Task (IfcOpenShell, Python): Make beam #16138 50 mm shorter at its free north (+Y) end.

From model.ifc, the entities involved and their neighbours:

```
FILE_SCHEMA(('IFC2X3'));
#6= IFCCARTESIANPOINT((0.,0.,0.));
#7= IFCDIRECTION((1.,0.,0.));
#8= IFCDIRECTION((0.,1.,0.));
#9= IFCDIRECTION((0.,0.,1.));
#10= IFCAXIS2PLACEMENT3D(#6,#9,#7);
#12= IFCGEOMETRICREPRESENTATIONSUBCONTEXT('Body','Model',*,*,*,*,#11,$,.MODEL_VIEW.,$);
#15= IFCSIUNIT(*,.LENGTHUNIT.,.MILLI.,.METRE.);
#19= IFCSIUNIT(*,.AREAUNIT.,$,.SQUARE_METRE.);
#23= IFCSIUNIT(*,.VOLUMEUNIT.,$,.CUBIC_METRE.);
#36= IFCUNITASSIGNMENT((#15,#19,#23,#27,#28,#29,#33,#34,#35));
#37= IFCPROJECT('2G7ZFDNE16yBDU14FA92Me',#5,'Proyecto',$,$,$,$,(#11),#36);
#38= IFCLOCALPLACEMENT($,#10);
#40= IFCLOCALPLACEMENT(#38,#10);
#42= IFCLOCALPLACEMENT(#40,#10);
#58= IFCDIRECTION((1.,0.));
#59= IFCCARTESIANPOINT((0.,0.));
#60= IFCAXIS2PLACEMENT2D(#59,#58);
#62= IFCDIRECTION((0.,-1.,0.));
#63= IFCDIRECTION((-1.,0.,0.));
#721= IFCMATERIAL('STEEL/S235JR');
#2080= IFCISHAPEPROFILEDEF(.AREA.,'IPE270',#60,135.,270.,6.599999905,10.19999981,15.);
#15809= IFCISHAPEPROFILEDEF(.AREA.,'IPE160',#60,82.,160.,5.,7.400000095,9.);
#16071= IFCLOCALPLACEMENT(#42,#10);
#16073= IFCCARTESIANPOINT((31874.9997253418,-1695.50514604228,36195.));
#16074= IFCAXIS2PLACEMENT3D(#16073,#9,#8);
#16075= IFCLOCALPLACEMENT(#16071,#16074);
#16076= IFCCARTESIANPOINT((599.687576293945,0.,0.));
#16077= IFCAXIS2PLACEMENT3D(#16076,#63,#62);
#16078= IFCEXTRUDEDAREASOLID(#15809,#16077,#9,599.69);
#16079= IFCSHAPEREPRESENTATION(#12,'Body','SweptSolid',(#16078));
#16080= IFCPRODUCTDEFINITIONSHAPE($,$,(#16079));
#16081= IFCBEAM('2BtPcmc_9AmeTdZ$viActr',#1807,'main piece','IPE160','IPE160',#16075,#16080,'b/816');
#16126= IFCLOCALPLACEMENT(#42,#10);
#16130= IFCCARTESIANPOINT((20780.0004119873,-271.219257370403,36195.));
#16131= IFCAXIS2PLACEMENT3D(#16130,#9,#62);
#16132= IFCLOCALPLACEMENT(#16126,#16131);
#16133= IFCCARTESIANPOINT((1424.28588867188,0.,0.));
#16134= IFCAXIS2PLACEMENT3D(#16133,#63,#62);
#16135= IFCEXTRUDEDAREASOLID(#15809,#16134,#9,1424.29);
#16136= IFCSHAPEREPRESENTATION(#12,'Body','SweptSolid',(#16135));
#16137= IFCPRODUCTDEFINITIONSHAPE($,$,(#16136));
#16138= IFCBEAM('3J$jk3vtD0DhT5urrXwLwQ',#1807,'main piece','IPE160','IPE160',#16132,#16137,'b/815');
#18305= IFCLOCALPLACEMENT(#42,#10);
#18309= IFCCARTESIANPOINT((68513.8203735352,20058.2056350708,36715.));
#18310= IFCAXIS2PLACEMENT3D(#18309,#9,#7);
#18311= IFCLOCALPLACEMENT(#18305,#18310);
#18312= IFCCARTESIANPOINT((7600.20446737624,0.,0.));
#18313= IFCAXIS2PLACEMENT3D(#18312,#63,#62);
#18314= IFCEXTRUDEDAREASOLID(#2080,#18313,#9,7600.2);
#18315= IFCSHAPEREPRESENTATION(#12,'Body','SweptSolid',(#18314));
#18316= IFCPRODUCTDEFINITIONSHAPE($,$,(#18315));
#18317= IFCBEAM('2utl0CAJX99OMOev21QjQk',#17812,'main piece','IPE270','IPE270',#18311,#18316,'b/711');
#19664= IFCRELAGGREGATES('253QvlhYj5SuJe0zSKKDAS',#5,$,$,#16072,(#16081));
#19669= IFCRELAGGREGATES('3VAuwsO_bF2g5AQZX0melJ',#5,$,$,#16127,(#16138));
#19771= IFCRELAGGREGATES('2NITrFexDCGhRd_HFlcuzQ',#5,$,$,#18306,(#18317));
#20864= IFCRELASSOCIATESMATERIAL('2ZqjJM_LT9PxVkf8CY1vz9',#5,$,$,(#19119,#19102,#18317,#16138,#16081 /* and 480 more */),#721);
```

```python
import ifcopenshell
import ifcopenshell.util.representation
import ifcopenshell.util.unit

model = ifcopenshell.open("model.ifc")
unit_scale = ifcopenshell.util.unit.calculate_unit_scale(model)

member = model.by_id(16138)
change = -0.05 / unit_scale

# The extrusion runs towards the end named, so only its depth changes.
body = ifcopenshell.util.representation.get_representation(member, "Model", "Body")
solid = body.Items[0]
old_length = solid.Depth
solid.Depth += change

print(f"length {old_length:g} -> {solid.Depth:g}")

model.write("model_rev.ifc")
```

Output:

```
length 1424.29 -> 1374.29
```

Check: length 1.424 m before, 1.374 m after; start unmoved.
